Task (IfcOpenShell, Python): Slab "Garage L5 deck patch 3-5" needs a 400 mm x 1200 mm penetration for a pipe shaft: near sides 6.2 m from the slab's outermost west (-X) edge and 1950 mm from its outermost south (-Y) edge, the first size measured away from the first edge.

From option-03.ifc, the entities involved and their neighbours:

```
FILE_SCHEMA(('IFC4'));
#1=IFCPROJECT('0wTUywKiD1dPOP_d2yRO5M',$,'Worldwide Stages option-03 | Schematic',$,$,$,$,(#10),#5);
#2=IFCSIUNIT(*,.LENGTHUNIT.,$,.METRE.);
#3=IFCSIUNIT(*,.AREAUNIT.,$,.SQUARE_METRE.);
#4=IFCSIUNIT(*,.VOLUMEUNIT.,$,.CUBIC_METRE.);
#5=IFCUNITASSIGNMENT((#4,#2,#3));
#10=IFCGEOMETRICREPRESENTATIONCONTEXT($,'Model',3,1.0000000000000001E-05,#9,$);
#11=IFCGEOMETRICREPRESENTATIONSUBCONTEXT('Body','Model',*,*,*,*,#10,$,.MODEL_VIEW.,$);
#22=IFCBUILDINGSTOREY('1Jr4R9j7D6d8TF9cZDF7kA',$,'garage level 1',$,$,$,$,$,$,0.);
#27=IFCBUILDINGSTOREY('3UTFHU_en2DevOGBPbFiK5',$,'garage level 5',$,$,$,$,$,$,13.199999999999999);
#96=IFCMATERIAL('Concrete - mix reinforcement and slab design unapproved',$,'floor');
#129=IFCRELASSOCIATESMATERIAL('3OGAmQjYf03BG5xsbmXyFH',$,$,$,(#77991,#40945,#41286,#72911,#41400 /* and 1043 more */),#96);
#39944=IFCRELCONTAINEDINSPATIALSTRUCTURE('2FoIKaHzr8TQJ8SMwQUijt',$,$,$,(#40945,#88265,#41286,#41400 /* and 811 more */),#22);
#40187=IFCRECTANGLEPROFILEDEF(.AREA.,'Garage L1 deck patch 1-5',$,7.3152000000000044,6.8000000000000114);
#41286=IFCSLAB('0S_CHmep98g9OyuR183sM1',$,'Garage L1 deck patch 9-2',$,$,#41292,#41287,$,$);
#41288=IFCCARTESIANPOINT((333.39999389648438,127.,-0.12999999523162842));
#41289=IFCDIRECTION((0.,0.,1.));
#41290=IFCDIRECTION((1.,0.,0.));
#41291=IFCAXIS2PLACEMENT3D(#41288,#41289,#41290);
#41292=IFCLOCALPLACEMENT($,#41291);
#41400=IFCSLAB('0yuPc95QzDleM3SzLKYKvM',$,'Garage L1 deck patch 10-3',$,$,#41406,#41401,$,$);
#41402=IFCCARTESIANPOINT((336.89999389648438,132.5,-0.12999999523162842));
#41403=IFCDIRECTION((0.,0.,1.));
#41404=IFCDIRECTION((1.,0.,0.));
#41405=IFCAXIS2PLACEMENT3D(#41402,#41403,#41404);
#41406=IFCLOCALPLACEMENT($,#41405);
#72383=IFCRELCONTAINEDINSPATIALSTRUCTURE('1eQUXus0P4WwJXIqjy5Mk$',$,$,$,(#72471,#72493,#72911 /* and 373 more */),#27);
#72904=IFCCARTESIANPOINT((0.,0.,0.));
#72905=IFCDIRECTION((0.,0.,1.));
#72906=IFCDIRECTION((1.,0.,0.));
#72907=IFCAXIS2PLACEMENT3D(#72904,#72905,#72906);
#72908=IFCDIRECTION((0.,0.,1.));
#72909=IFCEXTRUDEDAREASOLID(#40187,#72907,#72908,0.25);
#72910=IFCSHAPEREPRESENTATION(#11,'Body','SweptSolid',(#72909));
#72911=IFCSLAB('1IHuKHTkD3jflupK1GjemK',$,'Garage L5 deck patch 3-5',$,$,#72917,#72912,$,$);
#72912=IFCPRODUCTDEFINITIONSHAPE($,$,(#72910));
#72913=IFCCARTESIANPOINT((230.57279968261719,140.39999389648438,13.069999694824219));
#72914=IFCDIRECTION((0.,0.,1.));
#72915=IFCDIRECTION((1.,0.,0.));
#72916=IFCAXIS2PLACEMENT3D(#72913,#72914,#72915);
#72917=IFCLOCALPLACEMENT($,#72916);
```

```python
import numpy as np
import ifcopenshell
import ifcopenshell.api.feature
import ifcopenshell.api.geometry
import ifcopenshell.api.root
import ifcopenshell.geom
import ifcopenshell.util.placement
import ifcopenshell.util.representation
import ifcopenshell.util.shape
import ifcopenshell.util.unit

model = ifcopenshell.open("option-03.ifc")
unit_scale = ifcopenshell.util.unit.calculate_unit_scale(model)
settings = ifcopenshell.geom.settings()


def volume(element):
    """Net volume in cubic metres, openings subtracted."""
    shape = ifcopenshell.geom.create_shape(settings, element)
    return ifcopenshell.util.shape.get_volume(shape.geometry)


slab = model.by_id(72911)
before = volume(slab)

# Extent in the slab's own axes, in metres. The edges named are its -X and -Y sides.
slab_shape = ifcopenshell.geom.create_shape(settings, slab)
vertices = ifcopenshell.util.shape.get_vertices(slab_shape.geometry)
x_min, y_min, bottom = vertices.min(axis=0)
top = vertices[:, 2].max()

opening = ifcopenshell.api.root.create_entity(model, ifc_class="IfcOpeningElement", name="Pipe shaft opening", predefined_type="OPENING")
context = ifcopenshell.util.representation.get_context(model, "Model", "Body", "MODEL_VIEW")
width, depth = 0.4, 1.2
outline = [(0.0, 0.0), (width, 0.0), (width, depth), (0.0, depth), (0.0, 0.0)]
# Overshoot both faces by 50 mm so the cut is clean.
shape = ifcopenshell.api.geometry.add_slab_representation(
    model, context=context, depth=top - bottom + 0.1, polyline=outline
)
ifcopenshell.api.geometry.assign_representation(model, product=opening, representation=shape)

matrix = ifcopenshell.util.placement.get_local_placement(slab.ObjectPlacement)
matrix[:, 3] = matrix @ np.append(np.array([x_min + 6.2, y_min + 1.95, bottom - 0.05]) / unit_scale, 1.0)
ifcopenshell.api.geometry.edit_object_placement(model, product=opening, matrix=matrix, is_si=False)
ifcopenshell.api.feature.add_feature(model, feature=opening, element=slab)

after = volume(slab)

print(f"slab volume {before:.3f} -> {after:.3f} m3")

model.write("option-03_rev.ifc")
```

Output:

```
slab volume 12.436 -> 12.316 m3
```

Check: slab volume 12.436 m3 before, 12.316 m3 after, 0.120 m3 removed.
